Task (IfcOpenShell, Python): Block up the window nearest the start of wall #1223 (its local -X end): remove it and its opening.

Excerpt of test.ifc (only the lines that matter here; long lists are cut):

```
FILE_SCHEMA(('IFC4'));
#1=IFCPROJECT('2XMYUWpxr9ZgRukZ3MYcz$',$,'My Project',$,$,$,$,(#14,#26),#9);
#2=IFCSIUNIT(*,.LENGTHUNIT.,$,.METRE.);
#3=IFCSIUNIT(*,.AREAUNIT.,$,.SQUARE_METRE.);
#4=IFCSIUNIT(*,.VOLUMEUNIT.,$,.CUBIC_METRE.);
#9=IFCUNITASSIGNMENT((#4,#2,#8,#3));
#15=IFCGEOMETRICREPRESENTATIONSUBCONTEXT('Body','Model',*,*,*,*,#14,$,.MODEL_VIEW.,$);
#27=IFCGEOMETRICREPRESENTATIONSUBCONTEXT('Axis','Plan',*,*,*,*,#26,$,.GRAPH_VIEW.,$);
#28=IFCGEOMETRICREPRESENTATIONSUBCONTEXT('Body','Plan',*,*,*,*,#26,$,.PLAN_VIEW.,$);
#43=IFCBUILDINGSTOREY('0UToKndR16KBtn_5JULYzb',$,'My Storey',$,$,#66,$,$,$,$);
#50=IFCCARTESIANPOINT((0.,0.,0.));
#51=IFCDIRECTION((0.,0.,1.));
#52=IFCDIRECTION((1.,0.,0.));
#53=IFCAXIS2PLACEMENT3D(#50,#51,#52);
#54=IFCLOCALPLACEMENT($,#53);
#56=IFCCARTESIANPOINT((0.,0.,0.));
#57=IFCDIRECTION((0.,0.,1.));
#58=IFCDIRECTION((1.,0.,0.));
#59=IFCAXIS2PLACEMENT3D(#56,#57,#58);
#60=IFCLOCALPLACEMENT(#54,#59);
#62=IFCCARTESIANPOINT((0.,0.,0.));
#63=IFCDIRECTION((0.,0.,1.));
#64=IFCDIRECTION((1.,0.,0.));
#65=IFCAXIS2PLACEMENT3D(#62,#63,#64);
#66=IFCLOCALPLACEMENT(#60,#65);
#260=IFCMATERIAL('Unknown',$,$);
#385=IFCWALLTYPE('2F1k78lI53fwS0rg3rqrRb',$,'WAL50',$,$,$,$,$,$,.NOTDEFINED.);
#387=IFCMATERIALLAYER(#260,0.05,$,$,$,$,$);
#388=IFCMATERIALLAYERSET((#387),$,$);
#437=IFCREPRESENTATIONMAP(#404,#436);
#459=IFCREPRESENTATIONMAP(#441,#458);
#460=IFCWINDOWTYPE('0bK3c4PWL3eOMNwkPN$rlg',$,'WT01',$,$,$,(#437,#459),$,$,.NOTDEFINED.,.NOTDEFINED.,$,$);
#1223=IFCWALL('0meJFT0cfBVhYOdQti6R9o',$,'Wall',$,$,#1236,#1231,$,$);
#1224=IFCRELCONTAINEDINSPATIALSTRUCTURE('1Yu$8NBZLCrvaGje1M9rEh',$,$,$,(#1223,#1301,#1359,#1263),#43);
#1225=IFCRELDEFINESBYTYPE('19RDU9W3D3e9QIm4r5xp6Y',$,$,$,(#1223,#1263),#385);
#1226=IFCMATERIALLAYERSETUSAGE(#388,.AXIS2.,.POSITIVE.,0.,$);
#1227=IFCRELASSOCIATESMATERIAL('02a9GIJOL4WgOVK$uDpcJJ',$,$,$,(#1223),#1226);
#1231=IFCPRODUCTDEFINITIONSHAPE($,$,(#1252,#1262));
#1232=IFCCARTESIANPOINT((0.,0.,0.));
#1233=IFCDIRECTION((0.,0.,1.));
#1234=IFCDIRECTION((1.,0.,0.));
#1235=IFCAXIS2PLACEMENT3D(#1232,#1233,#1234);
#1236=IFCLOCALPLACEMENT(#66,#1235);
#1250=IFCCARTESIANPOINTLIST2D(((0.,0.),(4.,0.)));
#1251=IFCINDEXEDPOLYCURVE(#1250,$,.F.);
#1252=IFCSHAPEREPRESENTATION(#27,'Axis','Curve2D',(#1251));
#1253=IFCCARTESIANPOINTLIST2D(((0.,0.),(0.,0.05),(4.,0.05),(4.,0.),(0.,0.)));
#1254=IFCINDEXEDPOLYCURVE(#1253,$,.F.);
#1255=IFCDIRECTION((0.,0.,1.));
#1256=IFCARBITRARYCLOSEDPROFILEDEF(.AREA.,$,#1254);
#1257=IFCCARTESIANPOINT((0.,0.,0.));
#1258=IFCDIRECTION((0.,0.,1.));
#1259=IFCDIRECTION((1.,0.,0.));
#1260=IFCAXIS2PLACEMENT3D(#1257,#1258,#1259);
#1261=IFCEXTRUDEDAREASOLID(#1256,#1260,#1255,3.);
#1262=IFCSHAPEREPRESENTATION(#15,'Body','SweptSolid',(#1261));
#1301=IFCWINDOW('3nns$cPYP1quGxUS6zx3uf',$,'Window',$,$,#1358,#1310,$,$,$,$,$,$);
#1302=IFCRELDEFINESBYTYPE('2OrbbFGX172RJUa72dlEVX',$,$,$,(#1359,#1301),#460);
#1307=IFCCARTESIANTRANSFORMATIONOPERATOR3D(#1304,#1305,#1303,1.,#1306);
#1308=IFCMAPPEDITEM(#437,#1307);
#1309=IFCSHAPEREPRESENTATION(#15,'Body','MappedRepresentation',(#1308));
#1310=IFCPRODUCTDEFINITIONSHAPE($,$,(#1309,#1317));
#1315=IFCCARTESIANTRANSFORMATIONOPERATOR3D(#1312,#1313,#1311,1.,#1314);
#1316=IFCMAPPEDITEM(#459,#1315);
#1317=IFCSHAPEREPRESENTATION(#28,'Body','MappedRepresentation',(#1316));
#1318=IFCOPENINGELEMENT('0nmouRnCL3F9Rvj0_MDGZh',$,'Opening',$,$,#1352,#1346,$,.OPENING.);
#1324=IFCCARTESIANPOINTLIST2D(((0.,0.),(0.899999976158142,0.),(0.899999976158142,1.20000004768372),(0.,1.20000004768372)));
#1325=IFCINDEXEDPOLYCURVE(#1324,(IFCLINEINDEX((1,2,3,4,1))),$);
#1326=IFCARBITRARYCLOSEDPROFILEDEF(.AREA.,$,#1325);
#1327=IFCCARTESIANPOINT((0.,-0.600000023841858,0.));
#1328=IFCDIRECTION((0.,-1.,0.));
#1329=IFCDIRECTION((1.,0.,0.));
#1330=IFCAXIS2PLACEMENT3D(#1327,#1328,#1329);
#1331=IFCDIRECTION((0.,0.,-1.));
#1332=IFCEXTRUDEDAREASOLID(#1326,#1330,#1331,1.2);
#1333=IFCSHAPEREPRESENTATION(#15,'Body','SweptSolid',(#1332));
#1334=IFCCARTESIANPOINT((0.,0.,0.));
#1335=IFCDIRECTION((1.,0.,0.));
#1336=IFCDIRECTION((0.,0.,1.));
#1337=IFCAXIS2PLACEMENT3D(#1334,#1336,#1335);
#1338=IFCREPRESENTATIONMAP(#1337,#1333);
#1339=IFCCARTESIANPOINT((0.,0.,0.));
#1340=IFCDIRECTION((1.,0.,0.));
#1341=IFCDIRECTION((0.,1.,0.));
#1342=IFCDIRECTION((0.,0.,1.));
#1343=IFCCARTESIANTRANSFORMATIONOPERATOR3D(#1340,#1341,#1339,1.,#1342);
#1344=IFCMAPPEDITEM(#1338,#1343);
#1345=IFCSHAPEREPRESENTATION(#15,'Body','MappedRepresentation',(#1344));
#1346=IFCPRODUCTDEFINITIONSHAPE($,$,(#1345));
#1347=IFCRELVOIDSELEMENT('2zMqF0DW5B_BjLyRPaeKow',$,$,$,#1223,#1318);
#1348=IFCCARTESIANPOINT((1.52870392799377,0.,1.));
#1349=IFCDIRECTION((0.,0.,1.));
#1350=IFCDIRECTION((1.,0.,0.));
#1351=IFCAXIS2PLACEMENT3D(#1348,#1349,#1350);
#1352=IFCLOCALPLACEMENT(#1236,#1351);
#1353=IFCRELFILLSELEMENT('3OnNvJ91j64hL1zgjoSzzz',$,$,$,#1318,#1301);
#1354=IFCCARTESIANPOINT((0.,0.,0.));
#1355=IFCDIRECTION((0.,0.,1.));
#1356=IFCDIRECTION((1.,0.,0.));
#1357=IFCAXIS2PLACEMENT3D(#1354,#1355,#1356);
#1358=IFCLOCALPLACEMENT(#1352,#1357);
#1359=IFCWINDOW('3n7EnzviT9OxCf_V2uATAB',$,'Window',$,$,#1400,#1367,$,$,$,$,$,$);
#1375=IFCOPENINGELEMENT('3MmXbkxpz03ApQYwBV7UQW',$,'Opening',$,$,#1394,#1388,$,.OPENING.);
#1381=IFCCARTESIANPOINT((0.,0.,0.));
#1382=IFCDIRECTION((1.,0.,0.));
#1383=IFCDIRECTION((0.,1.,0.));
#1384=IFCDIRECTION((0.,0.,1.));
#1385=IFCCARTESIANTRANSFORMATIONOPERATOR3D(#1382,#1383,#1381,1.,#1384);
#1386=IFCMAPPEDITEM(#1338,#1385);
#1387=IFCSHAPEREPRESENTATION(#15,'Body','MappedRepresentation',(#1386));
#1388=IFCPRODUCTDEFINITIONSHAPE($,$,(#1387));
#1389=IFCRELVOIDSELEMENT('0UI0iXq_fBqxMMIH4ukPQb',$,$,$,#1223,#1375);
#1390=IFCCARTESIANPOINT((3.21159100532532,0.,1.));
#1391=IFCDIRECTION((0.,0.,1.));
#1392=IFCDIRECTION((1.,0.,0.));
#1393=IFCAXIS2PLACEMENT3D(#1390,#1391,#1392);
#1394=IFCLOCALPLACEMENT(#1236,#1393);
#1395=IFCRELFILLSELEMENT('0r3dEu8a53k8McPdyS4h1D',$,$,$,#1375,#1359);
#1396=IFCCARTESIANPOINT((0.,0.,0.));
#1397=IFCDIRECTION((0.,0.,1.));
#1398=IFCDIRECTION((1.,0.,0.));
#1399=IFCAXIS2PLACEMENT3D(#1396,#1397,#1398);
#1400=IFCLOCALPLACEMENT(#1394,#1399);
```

```python
import ifcopenshell
import ifcopenshell.api.feature
import ifcopenshell.api.root
import ifcopenshell.geom
import ifcopenshell.util.shape

model = ifcopenshell.open("test.ifc")
settings = ifcopenshell.geom.settings()


def volume(element):
    """Net volume in cubic metres, openings subtracted."""
    shape = ifcopenshell.geom.create_shape(settings, element)
    return ifcopenshell.util.shape.get_volume(shape.geometry)


window = model.by_id(1301)
opening = window.FillsVoids[0].RelatingOpeningElement
wall = opening.VoidsElements[0].RelatingBuildingElement
before = volume(wall)

ifcopenshell.api.root.remove_product(model, product=window)
ifcopenshell.api.feature.remove_feature(model, feature=opening)

after = volume(wall)

print(f"wall volume {before:.3f} -> {after:.3f} m3")

model.write("test_edited.ifc")
```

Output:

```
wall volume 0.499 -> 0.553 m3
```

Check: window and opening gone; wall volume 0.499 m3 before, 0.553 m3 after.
